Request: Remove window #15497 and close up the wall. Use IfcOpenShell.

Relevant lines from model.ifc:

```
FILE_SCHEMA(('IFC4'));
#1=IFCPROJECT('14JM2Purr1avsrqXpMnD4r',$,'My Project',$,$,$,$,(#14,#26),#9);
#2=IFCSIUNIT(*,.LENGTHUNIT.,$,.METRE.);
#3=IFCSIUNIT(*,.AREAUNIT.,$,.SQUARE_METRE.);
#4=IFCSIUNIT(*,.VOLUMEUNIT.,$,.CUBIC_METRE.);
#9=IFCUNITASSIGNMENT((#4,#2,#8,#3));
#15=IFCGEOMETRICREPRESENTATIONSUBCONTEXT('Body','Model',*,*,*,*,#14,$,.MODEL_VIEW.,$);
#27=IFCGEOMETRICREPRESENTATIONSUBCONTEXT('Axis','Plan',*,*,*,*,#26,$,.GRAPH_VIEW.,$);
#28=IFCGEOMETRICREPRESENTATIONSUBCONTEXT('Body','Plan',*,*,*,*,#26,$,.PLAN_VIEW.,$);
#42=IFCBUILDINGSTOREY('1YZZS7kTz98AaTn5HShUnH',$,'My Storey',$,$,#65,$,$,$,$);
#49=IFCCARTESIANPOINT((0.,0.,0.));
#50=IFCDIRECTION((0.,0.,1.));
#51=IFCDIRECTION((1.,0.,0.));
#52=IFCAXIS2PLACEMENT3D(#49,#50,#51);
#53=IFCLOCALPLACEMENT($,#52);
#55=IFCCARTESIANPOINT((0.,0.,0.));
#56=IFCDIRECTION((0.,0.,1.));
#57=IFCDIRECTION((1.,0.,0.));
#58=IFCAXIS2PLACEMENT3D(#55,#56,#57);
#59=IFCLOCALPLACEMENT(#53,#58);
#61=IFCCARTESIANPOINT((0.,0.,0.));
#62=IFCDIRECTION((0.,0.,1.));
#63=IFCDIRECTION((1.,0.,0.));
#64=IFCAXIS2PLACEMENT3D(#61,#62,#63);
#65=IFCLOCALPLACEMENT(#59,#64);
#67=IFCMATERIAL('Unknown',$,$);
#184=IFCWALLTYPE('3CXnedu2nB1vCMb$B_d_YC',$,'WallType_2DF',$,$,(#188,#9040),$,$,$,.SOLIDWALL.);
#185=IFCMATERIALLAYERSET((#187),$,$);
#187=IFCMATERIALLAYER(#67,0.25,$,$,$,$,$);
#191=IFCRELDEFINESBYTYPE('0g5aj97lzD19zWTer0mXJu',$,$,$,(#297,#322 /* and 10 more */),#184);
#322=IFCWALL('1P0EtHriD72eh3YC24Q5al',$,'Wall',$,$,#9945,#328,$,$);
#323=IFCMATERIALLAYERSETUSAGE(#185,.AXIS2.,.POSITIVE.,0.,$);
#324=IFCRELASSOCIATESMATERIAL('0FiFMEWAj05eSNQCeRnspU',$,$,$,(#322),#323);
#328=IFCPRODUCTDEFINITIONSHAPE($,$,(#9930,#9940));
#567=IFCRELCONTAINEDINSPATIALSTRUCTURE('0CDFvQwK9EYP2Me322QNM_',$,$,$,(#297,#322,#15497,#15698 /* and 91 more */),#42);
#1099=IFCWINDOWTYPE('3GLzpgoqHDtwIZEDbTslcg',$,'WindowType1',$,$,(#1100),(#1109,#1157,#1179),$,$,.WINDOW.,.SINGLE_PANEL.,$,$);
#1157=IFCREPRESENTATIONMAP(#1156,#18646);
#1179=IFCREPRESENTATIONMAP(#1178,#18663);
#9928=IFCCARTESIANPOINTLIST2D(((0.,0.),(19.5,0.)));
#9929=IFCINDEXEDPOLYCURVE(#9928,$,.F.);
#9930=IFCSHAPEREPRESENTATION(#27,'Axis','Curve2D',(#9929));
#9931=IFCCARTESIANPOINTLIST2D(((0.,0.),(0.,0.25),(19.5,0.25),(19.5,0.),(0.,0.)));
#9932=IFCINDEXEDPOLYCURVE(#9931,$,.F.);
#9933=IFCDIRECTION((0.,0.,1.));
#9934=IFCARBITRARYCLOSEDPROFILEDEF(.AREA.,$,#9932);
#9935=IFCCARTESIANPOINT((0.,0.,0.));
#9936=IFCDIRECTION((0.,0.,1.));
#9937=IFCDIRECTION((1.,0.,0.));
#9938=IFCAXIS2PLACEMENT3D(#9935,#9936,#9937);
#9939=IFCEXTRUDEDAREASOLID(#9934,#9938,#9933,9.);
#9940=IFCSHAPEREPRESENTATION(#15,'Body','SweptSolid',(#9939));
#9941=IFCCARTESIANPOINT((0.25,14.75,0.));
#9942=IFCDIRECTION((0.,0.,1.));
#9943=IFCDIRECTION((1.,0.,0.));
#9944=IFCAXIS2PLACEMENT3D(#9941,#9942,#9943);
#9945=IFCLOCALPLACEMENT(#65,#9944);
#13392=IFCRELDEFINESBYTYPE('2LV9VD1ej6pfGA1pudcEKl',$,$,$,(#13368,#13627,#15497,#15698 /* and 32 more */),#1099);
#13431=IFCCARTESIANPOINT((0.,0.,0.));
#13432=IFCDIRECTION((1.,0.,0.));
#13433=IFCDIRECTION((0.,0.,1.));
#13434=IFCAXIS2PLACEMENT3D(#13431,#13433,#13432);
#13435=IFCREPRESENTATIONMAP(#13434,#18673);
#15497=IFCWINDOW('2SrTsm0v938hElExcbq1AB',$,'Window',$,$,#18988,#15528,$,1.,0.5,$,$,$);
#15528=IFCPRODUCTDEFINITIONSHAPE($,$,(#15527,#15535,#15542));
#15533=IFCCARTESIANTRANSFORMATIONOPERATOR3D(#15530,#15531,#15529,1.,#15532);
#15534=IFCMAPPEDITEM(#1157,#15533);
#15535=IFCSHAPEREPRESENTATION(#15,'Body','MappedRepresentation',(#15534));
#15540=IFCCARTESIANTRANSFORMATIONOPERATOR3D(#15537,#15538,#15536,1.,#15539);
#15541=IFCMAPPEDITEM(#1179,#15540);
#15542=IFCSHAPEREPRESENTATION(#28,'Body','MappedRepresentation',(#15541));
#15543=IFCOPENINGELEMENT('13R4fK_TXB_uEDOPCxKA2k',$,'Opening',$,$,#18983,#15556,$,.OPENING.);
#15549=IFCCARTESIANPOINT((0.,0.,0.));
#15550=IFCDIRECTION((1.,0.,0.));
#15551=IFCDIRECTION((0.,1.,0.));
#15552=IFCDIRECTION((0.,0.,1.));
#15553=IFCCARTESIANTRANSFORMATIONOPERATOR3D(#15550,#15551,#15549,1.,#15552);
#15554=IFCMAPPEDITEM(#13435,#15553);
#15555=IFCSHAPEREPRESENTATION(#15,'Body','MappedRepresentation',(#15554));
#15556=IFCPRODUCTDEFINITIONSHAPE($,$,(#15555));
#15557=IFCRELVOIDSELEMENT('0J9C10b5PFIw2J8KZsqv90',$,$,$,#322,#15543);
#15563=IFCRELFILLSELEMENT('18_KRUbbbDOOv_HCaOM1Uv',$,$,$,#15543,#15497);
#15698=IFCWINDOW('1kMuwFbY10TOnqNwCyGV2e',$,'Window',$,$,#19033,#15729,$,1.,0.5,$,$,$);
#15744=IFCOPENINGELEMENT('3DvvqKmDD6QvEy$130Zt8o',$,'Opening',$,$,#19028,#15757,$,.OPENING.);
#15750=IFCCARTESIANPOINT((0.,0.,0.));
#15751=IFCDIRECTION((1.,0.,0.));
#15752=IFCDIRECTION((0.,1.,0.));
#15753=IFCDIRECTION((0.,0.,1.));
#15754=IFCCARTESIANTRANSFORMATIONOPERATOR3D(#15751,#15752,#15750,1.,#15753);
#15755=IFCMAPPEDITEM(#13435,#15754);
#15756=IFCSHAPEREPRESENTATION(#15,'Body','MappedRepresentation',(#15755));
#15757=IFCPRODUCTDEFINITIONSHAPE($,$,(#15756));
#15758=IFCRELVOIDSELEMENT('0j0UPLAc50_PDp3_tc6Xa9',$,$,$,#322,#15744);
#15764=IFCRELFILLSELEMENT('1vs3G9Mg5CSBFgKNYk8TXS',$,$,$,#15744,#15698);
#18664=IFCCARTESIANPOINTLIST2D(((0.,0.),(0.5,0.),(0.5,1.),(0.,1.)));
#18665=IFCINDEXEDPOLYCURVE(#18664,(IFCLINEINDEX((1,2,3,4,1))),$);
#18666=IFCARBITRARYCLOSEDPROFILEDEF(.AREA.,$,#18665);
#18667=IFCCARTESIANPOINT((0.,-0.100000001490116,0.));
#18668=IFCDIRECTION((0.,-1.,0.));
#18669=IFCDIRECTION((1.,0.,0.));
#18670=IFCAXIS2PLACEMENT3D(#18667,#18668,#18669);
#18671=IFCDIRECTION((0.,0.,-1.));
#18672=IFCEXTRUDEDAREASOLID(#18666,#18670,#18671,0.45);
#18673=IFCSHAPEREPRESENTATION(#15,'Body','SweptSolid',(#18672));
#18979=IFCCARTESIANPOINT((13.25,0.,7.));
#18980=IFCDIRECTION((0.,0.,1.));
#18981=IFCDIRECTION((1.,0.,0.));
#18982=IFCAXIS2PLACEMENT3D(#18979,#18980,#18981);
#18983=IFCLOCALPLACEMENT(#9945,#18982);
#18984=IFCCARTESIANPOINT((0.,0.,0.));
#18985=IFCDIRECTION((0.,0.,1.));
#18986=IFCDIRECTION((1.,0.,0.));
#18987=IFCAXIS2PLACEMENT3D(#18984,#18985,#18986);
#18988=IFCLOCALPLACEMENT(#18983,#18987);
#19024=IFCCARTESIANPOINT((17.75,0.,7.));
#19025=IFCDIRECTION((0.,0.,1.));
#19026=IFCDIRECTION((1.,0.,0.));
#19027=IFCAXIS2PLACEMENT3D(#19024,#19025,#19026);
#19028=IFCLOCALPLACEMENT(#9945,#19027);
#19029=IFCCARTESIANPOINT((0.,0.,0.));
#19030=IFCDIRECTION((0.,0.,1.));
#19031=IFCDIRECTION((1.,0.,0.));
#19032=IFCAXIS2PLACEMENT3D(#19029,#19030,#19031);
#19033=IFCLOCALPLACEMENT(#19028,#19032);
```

```python
import ifcopenshell
import ifcopenshell.api.feature
import ifcopenshell.api.root
import ifcopenshell.geom
import ifcopenshell.util.shape

model = ifcopenshell.open("model.ifc")
settings = ifcopenshell.geom.settings()


def volume(element):
    """Net volume in cubic metres, openings subtracted."""
    shape = ifcopenshell.geom.create_shape(settings, element)
    return ifcopenshell.util.shape.get_volume(shape.geometry)


window = model.by_guid("2SrTsm0v938hElExcbq1AB")
opening = window.FillsVoids[0].RelatingOpeningElement
wall = opening.VoidsElements[0].RelatingBuildingElement
before = volume(wall)

ifcopenshell.api.root.remove_product(model, product=window)
ifcopenshell.api.feature.remove_feature(model, feature=opening)

after = volume(wall)

print(f"wall volume {before:.3f} -> {after:.3f} m3")

model.write("model_edited.ifc")
```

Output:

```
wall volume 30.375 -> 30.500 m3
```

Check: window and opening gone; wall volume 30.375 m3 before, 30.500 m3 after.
